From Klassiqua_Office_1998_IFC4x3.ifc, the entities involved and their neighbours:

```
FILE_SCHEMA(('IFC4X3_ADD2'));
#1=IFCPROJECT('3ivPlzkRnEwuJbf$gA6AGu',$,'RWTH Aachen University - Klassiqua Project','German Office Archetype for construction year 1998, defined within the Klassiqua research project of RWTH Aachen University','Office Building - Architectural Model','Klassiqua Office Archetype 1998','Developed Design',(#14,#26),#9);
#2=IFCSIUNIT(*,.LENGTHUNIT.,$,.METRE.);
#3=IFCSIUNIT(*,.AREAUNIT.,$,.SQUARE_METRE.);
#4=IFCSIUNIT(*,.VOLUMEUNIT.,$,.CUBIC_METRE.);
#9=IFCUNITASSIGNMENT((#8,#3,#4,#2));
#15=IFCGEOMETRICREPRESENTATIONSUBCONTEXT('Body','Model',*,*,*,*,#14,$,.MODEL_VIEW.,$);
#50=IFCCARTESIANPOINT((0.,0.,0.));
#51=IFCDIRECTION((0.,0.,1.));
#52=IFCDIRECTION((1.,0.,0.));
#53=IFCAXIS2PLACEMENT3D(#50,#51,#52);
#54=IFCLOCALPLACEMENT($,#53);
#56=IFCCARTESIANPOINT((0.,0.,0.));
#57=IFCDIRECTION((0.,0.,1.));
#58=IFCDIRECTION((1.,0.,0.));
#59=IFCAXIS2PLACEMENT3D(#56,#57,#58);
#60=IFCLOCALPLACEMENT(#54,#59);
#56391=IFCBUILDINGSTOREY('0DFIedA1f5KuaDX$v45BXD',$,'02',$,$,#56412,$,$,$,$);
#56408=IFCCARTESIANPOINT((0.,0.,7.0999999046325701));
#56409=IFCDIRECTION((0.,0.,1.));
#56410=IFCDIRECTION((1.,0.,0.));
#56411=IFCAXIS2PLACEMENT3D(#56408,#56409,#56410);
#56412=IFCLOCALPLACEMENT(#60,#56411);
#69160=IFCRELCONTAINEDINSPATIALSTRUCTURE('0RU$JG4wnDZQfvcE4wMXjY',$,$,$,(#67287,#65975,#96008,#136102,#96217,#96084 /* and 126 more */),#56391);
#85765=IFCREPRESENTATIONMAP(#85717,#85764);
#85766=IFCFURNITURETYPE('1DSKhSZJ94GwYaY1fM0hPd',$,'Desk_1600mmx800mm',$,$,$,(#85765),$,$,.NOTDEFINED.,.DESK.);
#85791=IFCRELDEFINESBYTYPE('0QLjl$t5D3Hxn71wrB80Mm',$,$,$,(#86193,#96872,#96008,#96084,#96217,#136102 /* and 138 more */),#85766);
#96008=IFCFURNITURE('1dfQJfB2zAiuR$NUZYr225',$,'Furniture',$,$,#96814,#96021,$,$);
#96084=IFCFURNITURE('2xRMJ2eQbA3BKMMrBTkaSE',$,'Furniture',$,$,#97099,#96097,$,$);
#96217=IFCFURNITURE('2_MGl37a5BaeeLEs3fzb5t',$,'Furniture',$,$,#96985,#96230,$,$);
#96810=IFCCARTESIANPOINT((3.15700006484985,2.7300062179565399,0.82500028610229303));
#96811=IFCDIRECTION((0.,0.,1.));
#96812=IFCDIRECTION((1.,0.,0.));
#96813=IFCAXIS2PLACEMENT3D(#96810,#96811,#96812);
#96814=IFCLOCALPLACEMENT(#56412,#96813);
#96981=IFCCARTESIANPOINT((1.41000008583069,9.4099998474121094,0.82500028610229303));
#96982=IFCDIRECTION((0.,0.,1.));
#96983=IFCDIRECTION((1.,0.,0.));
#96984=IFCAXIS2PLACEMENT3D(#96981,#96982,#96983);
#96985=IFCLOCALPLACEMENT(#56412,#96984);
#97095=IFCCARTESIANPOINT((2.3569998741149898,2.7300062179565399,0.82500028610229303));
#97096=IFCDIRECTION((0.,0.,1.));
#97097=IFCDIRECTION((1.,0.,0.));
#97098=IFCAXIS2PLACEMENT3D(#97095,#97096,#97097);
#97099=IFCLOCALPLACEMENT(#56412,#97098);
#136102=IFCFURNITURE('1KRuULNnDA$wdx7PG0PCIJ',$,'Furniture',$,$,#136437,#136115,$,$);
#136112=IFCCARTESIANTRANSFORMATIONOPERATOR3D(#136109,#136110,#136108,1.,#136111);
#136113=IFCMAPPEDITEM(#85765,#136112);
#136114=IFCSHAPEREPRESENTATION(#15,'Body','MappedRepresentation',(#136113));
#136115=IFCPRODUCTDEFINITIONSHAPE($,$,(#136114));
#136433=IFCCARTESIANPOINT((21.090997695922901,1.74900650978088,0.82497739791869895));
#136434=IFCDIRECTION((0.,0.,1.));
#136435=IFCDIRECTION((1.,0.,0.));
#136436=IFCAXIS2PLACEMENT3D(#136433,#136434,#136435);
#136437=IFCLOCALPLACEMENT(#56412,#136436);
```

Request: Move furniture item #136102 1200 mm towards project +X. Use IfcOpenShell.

```python
import ifcopenshell
import ifcopenshell.api.geometry
import ifcopenshell.util.placement

model = ifcopenshell.open("Klassiqua_Office_1998_IFC4x3.ifc")

item = model.by_guid("1KRuULNnDA$wdx7PG0PCIJ")
matrix = ifcopenshell.util.placement.get_local_placement(item.ObjectPlacement)
matrix[0, 3] += 1.2
ifcopenshell.api.geometry.edit_object_placement(model, product=item, matrix=matrix, is_si=False)

print(ifcopenshell.util.placement.get_local_placement(item.ObjectPlacement).round(3) + 0.0)

model.write("Klassiqua_Office_1998_IFC4x3_rev.ifc")
```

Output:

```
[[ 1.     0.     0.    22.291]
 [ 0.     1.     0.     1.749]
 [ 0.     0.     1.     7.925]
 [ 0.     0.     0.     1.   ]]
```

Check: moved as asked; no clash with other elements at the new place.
